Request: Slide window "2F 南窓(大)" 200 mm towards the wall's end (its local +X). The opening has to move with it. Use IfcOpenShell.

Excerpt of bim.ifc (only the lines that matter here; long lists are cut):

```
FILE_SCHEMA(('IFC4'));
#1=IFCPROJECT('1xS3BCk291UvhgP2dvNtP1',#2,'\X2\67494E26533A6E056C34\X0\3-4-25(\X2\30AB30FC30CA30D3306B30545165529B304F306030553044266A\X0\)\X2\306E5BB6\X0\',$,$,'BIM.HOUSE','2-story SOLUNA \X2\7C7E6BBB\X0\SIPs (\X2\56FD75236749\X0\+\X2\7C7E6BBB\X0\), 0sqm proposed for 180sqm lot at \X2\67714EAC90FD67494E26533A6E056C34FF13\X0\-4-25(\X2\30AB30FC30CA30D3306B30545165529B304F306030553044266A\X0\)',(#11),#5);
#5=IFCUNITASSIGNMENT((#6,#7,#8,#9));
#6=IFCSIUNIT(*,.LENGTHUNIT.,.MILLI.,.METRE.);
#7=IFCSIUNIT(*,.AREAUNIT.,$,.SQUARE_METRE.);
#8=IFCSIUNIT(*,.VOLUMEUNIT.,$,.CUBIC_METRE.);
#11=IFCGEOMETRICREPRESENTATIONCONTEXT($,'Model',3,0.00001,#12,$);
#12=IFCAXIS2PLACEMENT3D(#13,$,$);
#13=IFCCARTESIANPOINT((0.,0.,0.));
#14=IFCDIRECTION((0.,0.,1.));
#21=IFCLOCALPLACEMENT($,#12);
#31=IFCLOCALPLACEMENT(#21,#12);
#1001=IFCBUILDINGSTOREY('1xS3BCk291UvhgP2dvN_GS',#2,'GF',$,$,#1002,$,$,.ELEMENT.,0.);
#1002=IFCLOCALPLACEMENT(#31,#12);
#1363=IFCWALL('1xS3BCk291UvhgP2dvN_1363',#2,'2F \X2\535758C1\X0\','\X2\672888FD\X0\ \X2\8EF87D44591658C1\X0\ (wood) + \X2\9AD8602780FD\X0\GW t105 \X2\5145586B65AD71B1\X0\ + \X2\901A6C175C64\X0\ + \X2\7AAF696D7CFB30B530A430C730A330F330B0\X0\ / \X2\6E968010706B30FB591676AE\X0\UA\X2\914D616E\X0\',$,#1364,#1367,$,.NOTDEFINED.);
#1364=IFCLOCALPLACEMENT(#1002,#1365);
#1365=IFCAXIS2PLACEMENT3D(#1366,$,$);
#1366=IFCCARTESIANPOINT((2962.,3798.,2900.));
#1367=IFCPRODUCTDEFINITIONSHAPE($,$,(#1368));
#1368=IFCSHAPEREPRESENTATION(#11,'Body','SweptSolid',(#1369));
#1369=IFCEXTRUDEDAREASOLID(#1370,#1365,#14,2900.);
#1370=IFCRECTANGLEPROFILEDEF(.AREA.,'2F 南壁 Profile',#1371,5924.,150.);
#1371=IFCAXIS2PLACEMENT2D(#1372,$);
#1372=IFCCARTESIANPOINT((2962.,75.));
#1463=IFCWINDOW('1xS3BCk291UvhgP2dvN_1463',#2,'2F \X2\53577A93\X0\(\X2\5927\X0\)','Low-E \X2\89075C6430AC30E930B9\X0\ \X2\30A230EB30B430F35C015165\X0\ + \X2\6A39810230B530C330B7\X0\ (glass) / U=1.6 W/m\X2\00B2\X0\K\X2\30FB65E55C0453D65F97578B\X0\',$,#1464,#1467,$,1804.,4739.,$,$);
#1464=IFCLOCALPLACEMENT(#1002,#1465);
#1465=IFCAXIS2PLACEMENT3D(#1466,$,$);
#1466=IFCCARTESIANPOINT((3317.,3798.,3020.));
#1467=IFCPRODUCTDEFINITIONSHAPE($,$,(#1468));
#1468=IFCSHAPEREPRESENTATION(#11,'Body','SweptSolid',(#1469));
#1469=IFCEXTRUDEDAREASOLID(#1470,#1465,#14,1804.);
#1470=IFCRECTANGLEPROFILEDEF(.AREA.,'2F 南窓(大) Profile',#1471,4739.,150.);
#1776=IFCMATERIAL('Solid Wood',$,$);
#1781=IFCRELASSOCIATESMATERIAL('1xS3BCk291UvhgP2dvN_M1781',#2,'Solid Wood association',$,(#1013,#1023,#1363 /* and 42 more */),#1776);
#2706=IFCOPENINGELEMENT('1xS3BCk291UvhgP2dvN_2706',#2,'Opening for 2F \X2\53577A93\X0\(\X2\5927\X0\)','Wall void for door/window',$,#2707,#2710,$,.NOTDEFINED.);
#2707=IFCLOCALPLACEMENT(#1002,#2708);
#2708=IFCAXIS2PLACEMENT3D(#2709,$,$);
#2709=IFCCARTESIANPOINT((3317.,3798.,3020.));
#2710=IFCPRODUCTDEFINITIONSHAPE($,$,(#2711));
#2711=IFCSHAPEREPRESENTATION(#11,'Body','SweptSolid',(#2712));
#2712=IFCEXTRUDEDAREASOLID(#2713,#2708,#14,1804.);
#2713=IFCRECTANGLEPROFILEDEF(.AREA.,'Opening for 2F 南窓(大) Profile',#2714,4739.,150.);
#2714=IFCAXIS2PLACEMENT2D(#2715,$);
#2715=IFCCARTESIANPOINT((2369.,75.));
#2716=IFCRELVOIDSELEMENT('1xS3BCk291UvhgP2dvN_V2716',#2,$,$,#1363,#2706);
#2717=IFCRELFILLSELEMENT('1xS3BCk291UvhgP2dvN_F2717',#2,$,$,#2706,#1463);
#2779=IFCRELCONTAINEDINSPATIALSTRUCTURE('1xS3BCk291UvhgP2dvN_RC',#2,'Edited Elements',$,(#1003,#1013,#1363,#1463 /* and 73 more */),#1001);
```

```python
import ifcopenshell
import ifcopenshell.api.geometry
import ifcopenshell.util.placement
import ifcopenshell.util.unit

model = ifcopenshell.open("bim.ifc")
unit_scale = ifcopenshell.util.unit.calculate_unit_scale(model)

window = model.by_guid("1xS3BCk291UvhgP2dvN_1463")
opening = window.FillsVoids[0].RelatingOpeningElement
wall = opening.VoidsElements[0].RelatingBuildingElement

wall_matrix = ifcopenshell.util.placement.get_local_placement(wall.ObjectPlacement)
shift = wall_matrix[:3, 0] * 0.2 / unit_scale
before = ifcopenshell.util.placement.get_local_placement(window.ObjectPlacement)[:3, 3].copy()

# The window is not placed relative to its opening, so move both.
for product in (opening, window):
    matrix = ifcopenshell.util.placement.get_local_placement(product.ObjectPlacement)
    matrix[:3, 3] += shift
    ifcopenshell.api.geometry.edit_object_placement(model, product=product, matrix=matrix, is_si=False)

after = ifcopenshell.util.placement.get_local_placement(window.ObjectPlacement)[:3, 3]
print("window moved by", (after - before).round(3) + 0.0)

model.write("bim_edited.ifc")
```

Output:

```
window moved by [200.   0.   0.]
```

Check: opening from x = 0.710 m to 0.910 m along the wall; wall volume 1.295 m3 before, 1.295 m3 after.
